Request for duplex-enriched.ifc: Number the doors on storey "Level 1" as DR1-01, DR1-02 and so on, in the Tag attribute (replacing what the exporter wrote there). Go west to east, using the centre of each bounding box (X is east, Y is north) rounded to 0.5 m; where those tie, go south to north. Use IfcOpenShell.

First a look at what the model holds.

```python
import ifcopenshell
import ifcopenshell.util.element
import ifcopenshell.util.placement

model = ifcopenshell.open("duplex-enriched.ifc")
print(model.schema)
storey = next(s for s in model.by_type("IfcBuildingStorey") if s.Name == "Level 1")
doors = [e for e in ifcopenshell.util.element.get_decomposition(storey) if e.is_a("IfcDoor")]
for e in sorted(doors, key=lambda e: e.id()):
    origin = ifcopenshell.util.placement.get_local_placement(e.ObjectPlacement)[:3, 3]
    print(e.id(), e.Tag, e.Name, origin.round(2) + 0.0, sep=" | ")
```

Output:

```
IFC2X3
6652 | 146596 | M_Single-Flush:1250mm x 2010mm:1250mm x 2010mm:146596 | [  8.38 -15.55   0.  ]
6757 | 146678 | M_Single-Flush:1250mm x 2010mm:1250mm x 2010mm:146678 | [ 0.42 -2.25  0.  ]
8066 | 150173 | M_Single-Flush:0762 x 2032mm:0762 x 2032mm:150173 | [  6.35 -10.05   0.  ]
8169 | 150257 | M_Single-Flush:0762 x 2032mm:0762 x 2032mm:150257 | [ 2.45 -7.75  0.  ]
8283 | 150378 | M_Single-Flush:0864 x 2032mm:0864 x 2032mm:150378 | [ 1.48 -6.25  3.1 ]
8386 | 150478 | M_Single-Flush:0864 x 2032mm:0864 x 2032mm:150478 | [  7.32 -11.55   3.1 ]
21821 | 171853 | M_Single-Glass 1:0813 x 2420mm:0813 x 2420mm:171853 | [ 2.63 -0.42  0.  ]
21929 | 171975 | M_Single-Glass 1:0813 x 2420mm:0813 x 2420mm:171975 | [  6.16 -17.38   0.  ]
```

```python
import ifcopenshell
import ifcopenshell.geom
import ifcopenshell.util.element
import ifcopenshell.util.shape

model = ifcopenshell.open("duplex-enriched.ifc")
settings = ifcopenshell.geom.settings()
settings.set("use-world-coords", True)


def centre(element):
    shape = ifcopenshell.geom.create_shape(settings, element)
    return ifcopenshell.util.shape.get_bbox_centroid(shape.geometry)


storey = next(s for s in model.by_type("IfcBuildingStorey") if s.Name == "Level 1")
doors = [e for e in ifcopenshell.util.element.get_decomposition(storey) if e.is_a("IfcDoor")]

# Insertion points can sit at a corner or the storey origin, so sort by the geometry (in metres).
centres = {e: centre(e) for e in doors}
doors.sort(key=lambda e: (round(centres[e][0] / 0.5), centres[e][1]))

for i, e in enumerate(doors, start=1):
    number = f"DR1-{i:02d}"
    e.Tag = number
    print(e.id(), number)

model.write("duplex-enriched-out.ifc")
```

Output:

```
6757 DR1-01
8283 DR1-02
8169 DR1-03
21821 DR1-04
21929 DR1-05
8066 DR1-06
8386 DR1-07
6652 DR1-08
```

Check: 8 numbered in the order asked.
